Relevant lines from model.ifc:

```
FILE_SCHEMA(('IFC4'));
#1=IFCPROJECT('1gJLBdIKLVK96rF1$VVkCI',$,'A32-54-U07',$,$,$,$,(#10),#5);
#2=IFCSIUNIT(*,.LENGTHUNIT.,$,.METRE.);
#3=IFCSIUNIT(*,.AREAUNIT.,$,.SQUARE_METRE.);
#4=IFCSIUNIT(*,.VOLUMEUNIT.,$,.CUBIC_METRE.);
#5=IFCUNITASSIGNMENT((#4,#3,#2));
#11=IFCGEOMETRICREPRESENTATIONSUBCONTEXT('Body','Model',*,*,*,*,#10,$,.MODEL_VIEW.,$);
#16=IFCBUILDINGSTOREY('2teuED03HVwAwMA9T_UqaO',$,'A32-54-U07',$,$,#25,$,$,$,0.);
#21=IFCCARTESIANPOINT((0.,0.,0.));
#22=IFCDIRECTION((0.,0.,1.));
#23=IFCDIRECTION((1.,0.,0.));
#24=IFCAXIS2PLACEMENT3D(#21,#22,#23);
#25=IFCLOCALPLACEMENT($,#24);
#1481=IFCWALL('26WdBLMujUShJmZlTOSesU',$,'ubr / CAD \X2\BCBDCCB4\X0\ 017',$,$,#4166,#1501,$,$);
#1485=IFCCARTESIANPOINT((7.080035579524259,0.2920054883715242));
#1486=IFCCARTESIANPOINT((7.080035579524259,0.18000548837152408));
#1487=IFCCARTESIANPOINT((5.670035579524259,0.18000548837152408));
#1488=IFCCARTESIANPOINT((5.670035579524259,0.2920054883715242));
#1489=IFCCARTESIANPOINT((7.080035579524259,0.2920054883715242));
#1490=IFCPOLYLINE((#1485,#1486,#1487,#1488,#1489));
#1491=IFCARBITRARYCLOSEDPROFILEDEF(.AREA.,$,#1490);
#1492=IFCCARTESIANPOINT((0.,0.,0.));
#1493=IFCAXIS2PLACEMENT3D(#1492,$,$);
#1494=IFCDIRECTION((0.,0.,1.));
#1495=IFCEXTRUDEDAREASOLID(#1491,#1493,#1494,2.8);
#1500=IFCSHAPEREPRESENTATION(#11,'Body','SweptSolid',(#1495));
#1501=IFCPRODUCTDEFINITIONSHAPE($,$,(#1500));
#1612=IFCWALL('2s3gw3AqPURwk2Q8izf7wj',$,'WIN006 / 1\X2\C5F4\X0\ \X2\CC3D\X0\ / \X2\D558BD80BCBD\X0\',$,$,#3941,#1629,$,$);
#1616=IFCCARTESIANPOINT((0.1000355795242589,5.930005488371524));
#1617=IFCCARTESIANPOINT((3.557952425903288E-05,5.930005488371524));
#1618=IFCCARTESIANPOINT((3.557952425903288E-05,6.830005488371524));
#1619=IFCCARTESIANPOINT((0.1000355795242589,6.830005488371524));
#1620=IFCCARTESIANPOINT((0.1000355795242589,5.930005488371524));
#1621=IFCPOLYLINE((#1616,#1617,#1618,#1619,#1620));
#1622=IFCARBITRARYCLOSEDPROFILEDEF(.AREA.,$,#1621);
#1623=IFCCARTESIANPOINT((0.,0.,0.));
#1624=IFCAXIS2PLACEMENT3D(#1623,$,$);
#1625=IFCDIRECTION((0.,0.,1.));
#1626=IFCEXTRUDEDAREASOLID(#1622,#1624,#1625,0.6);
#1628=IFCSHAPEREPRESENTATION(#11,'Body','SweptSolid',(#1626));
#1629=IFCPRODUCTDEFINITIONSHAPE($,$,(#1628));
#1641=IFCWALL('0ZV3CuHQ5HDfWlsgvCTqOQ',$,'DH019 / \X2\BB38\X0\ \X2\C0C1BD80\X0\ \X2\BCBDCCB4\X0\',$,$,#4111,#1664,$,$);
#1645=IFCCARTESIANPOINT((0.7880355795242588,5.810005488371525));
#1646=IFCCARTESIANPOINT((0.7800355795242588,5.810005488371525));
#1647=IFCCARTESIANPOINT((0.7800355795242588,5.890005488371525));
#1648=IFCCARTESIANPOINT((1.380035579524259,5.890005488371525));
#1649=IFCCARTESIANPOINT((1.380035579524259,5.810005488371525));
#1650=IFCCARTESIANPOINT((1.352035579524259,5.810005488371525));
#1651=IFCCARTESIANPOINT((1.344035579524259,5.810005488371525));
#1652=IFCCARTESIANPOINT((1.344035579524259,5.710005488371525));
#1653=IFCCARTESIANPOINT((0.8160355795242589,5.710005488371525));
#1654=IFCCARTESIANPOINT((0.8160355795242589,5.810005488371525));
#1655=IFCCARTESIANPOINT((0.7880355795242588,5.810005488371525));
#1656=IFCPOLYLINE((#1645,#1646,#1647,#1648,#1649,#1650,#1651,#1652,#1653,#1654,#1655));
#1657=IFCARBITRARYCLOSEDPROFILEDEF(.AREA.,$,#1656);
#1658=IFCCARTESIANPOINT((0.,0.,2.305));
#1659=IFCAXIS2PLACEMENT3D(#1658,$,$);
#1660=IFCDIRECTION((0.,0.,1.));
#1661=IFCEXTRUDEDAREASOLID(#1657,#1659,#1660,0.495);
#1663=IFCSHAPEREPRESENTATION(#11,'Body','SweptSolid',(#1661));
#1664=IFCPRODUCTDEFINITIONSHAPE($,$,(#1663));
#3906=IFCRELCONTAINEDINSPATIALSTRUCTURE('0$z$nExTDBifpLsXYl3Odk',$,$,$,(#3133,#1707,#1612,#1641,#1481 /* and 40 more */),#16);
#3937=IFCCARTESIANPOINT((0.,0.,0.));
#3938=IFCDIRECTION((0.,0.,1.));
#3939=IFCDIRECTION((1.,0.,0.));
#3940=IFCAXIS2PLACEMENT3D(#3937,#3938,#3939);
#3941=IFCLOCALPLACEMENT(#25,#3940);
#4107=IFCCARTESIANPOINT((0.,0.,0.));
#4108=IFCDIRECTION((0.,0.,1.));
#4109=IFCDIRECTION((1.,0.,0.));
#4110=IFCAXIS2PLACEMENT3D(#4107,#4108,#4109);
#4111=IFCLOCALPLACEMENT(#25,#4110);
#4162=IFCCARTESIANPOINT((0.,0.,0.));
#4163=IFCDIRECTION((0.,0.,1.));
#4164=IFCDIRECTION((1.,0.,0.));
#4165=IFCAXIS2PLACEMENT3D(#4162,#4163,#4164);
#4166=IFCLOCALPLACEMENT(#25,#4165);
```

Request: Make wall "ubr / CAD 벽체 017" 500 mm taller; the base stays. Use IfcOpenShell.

```python
import ifcopenshell
import ifcopenshell.geom
import ifcopenshell.util.representation
import ifcopenshell.util.shape
import ifcopenshell.util.unit

model = ifcopenshell.open("model.ifc")
unit_scale = ifcopenshell.util.unit.calculate_unit_scale(model)
settings = ifcopenshell.geom.settings()


def volume(element):
    """Net volume in cubic metres, openings subtracted."""
    shape = ifcopenshell.geom.create_shape(settings, element)
    return ifcopenshell.util.shape.get_volume(shape.geometry)


wall = model.by_guid("26WdBLMujUShJmZlTOSesU")
before = volume(wall)

body = ifcopenshell.util.representation.get_representation(wall, "Model", "Body")
solid = body.Items[0]
old_height = solid.Depth
solid.Depth += 0.5 / unit_scale
after = volume(wall)

print(f"height {old_height:g} -> {solid.Depth:g}, volume {before:.3f} -> {after:.3f} m3")

model.write("model_v2.ifc")
```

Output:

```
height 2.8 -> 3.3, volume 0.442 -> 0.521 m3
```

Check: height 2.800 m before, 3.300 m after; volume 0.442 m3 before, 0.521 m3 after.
